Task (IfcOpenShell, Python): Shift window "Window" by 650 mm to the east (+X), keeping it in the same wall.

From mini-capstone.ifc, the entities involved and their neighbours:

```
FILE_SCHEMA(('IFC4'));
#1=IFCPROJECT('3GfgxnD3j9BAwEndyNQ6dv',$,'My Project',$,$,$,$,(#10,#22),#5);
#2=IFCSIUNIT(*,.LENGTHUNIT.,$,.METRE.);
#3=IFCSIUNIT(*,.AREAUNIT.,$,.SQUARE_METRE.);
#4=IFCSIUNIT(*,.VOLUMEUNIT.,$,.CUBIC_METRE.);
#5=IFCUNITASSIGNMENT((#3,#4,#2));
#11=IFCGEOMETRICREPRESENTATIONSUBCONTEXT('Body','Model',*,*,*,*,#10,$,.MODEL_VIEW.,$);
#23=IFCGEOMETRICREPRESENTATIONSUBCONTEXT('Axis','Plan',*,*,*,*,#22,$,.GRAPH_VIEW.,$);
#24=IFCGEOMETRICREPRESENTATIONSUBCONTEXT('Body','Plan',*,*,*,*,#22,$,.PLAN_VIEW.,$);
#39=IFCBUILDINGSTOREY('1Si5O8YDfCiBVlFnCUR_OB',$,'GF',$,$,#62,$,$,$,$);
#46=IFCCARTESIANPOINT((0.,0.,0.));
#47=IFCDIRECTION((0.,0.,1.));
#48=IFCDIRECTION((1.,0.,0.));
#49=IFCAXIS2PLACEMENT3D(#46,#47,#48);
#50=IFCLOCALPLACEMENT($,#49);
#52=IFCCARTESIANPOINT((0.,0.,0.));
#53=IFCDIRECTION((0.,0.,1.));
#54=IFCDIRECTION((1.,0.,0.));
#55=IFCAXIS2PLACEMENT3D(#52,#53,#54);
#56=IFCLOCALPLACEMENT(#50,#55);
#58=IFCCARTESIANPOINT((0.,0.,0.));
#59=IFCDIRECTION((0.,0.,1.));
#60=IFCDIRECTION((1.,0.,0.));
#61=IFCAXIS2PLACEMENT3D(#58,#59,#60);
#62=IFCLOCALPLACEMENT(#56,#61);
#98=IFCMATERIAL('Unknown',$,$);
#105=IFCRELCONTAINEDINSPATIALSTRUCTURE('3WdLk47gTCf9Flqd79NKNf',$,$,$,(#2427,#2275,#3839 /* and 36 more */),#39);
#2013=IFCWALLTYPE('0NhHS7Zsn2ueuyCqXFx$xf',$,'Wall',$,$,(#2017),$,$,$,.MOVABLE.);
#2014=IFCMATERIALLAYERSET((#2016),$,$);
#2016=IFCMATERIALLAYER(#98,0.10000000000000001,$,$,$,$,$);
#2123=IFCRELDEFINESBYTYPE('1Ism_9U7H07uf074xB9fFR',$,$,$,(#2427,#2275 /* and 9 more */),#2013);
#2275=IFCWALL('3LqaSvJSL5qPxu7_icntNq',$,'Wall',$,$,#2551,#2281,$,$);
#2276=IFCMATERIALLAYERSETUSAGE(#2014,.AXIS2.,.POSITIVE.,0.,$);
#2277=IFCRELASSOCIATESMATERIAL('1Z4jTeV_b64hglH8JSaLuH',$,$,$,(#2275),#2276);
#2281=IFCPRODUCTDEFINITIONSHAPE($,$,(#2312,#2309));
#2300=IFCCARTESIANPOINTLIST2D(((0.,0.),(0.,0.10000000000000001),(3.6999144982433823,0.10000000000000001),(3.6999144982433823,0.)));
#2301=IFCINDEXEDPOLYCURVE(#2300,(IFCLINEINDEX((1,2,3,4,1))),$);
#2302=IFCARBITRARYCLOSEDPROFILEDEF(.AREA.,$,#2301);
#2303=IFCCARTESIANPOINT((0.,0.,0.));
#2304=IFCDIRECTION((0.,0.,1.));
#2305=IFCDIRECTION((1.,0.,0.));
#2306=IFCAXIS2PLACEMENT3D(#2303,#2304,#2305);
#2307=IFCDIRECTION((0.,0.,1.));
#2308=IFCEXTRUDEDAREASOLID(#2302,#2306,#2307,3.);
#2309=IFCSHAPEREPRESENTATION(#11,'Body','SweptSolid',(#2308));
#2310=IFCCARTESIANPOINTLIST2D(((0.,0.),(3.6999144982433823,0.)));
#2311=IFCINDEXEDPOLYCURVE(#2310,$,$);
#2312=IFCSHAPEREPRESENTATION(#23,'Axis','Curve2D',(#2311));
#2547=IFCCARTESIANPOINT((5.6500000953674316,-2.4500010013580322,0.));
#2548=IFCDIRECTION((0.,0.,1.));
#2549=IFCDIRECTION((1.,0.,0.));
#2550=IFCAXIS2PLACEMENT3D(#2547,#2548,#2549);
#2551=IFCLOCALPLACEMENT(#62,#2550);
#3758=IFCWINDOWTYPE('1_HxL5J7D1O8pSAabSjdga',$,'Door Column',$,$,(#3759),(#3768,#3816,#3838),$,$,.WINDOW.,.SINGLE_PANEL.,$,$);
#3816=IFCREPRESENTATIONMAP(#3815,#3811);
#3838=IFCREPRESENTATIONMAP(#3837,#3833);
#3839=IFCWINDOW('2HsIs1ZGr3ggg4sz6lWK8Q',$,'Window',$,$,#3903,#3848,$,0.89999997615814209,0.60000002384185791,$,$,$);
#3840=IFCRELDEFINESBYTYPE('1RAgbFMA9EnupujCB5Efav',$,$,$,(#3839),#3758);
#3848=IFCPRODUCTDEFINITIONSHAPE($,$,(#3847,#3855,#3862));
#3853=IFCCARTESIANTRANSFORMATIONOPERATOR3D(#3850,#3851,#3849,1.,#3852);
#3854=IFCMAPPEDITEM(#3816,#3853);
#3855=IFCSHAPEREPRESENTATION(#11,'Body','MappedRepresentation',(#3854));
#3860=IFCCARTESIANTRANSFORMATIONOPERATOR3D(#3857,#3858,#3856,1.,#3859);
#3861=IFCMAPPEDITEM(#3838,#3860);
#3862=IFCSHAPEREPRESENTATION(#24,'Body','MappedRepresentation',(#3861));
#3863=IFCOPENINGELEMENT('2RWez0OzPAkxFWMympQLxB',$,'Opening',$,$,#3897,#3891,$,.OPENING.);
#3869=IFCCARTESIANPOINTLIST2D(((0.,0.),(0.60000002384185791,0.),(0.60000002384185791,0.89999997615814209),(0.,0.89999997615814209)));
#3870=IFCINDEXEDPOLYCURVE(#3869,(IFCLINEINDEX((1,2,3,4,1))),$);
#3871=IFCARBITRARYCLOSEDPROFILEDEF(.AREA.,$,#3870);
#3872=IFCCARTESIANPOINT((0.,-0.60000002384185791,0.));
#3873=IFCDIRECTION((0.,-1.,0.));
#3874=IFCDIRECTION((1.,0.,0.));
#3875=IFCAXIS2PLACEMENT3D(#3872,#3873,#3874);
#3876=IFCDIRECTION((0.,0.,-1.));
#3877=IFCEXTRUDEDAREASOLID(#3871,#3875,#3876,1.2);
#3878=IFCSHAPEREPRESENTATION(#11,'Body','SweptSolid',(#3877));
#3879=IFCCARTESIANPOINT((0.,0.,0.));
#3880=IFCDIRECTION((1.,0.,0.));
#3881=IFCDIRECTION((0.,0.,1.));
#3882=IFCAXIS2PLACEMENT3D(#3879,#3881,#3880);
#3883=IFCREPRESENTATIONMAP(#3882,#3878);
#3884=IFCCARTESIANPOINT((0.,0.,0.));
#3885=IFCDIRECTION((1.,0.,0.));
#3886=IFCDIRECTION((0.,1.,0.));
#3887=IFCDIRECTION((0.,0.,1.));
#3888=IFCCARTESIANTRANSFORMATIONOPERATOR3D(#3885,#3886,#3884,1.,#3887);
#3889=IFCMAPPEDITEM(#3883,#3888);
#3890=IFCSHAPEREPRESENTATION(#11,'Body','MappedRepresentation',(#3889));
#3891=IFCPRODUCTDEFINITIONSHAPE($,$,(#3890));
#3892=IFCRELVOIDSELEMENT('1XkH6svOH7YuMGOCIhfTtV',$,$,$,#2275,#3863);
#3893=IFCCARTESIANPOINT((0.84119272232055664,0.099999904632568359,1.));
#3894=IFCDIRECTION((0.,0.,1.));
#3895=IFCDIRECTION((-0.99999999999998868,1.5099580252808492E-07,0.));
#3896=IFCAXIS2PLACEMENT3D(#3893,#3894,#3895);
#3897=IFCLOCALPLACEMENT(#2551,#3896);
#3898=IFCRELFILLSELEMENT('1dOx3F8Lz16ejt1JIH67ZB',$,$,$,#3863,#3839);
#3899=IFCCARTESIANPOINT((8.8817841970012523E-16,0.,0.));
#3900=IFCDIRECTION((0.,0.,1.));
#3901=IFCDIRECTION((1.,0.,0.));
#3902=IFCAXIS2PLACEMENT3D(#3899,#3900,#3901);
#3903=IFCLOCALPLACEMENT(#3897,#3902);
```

```python
import ifcopenshell
import ifcopenshell.api.geometry
import ifcopenshell.util.placement

model = ifcopenshell.open("mini-capstone.ifc")

window = model.by_guid("2HsIs1ZGr3ggg4sz6lWK8Q")
opening = window.FillsVoids[0].RelatingOpeningElement
wall = opening.VoidsElements[0].RelatingBuildingElement

wall_matrix = ifcopenshell.util.placement.get_local_placement(wall.ObjectPlacement)
shift = wall_matrix[:3, 0] * 0.65
before = ifcopenshell.util.placement.get_local_placement(window.ObjectPlacement)[:3, 3].copy()

# The window is placed relative to its opening, so it follows when the opening moves.
matrix = ifcopenshell.util.placement.get_local_placement(opening.ObjectPlacement)
matrix[:3, 3] += shift
ifcopenshell.api.geometry.edit_object_placement(
    model, product=opening, matrix=matrix, is_si=False, should_transform_children=True
)

after = ifcopenshell.util.placement.get_local_placement(window.ObjectPlacement)[:3, 3]
print("window moved by", (after - before).round(3) + 0.0)

model.write("mini-capstone-out.ifc")
```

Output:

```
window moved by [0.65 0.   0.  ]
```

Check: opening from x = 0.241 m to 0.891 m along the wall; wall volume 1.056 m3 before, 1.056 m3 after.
